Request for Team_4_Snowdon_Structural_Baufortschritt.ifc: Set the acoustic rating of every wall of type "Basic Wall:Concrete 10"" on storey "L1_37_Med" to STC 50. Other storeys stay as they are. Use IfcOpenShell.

First a look at what the model holds.

```python
import ifcopenshell
import ifcopenshell.util.element

model = ifcopenshell.open("Team_4_Snowdon_Structural_Baufortschritt.ifc")
print(model.schema)
storey = next(s for s in model.by_type("IfcBuildingStorey") if s.Name == "L1_37_Med")
walls = [e for e in ifcopenshell.util.element.get_decomposition(storey) if e.is_a("IfcWall")]
seen = {}
for e in walls:
    element_type = ifcopenshell.util.element.get_type(e)
    key = (element_type.Name if element_type != e and element_type else None, ifcopenshell.util.element.get_pset(e, "Pset_WallCommon", "AcousticRating"))
    seen[key] = seen.get(key, 0) + 1
for (name, value), count in sorted(seen.items(), key=str):
    print(count, "x", name, "|", value)
```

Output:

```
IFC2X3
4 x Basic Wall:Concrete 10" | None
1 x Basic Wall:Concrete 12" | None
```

```python
import ifcopenshell
import ifcopenshell.api.pset
import ifcopenshell.util.element

model = ifcopenshell.open("Team_4_Snowdon_Structural_Baufortschritt.ifc")

storey = next(s for s in model.by_type("IfcBuildingStorey") if s.Name == "L1_37_Med")
walls = [e for e in ifcopenshell.util.element.get_decomposition(storey) if e.is_a("IfcWall")]

count = 0
for e in walls:
    element_type = ifcopenshell.util.element.get_type(e)
    if element_type in (None, e) or element_type.Name != 'Basic Wall:Concrete 10"':
        continue
    # add_pset returns the element's existing set when there is one.
    pset = ifcopenshell.api.pset.add_pset(model, product=e, name="Pset_WallCommon")
    ifcopenshell.api.pset.edit_pset(model, pset=pset, properties={"AcousticRating": "STC 50"})
    count += 1

print(count, "walls updated")

model.write("Team_4_Snowdon_Structural_Baufortschritt_rev.ifc")
```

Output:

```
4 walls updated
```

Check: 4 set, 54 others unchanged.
